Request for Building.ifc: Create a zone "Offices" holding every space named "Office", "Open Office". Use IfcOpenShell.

First a look at what the model holds.

```python
import ifcopenshell

model = ifcopenshell.open("Building.ifc")
print(model.schema)
seen = {}
for space in model.by_type("IfcSpace"):
    seen[space.LongName] = seen.get(space.LongName, 0) + 1
for name, count in sorted(seen.items(), key=str):
    print(count, "x", name)
print("zones:", [z.Name for z in model.by_type("IfcZone")][:20])
```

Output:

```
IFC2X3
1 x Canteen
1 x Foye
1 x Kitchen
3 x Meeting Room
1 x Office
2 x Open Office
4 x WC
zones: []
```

```python
import ifcopenshell
import ifcopenshell.api.group
import ifcopenshell.api.root

model = ifcopenshell.open("Building.ifc")

names = {"Office", "Open Office"}
spaces = [s for s in model.by_type("IfcSpace") if s.LongName in names]

zone = ifcopenshell.api.root.create_entity(model, ifc_class="IfcZone", name="Offices")
ifcopenshell.api.group.assign_group(model, products=spaces, group=zone)
print(len(spaces), "spaces in", zone.Name)

model.write("Building_updated.ifc")
```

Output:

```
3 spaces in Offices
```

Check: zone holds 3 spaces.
